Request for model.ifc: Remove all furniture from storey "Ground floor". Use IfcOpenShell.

First a look at what the model holds.

```python
import ifcopenshell
import ifcopenshell.util.element

model = ifcopenshell.open("model.ifc")
print(model.schema)
storey = next(s for s in model.by_type("IfcBuildingStorey") if s.Name == "Ground floor")
furniture = [e for e in ifcopenshell.util.element.get_decomposition(storey) if e.is_a("IfcFurnishingElement")]
seen = {}
for e in furniture:
    element_type = ifcopenshell.util.element.get_type(e)
    name = element_type.Name if element_type not in (None, e) else None
    seen[name] = seen.get(name, 0) + 1
for name, count in sorted(seen.items(), key=str):
    print(count, "x", name)
```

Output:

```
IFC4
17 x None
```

```python
import ifcopenshell
import ifcopenshell.api.root
import ifcopenshell.util.element

model = ifcopenshell.open("model.ifc")

storey = next(s for s in model.by_type("IfcBuildingStorey") if s.Name == "Ground floor")
furniture = [e for e in ifcopenshell.util.element.get_decomposition(storey) if e.is_a("IfcFurnishingElement")]

for e in furniture:
    ifcopenshell.api.root.remove_product(model, product=e)
print(len(furniture), "removed")

model.write("model-out.ifc")
```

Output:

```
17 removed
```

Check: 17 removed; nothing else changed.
